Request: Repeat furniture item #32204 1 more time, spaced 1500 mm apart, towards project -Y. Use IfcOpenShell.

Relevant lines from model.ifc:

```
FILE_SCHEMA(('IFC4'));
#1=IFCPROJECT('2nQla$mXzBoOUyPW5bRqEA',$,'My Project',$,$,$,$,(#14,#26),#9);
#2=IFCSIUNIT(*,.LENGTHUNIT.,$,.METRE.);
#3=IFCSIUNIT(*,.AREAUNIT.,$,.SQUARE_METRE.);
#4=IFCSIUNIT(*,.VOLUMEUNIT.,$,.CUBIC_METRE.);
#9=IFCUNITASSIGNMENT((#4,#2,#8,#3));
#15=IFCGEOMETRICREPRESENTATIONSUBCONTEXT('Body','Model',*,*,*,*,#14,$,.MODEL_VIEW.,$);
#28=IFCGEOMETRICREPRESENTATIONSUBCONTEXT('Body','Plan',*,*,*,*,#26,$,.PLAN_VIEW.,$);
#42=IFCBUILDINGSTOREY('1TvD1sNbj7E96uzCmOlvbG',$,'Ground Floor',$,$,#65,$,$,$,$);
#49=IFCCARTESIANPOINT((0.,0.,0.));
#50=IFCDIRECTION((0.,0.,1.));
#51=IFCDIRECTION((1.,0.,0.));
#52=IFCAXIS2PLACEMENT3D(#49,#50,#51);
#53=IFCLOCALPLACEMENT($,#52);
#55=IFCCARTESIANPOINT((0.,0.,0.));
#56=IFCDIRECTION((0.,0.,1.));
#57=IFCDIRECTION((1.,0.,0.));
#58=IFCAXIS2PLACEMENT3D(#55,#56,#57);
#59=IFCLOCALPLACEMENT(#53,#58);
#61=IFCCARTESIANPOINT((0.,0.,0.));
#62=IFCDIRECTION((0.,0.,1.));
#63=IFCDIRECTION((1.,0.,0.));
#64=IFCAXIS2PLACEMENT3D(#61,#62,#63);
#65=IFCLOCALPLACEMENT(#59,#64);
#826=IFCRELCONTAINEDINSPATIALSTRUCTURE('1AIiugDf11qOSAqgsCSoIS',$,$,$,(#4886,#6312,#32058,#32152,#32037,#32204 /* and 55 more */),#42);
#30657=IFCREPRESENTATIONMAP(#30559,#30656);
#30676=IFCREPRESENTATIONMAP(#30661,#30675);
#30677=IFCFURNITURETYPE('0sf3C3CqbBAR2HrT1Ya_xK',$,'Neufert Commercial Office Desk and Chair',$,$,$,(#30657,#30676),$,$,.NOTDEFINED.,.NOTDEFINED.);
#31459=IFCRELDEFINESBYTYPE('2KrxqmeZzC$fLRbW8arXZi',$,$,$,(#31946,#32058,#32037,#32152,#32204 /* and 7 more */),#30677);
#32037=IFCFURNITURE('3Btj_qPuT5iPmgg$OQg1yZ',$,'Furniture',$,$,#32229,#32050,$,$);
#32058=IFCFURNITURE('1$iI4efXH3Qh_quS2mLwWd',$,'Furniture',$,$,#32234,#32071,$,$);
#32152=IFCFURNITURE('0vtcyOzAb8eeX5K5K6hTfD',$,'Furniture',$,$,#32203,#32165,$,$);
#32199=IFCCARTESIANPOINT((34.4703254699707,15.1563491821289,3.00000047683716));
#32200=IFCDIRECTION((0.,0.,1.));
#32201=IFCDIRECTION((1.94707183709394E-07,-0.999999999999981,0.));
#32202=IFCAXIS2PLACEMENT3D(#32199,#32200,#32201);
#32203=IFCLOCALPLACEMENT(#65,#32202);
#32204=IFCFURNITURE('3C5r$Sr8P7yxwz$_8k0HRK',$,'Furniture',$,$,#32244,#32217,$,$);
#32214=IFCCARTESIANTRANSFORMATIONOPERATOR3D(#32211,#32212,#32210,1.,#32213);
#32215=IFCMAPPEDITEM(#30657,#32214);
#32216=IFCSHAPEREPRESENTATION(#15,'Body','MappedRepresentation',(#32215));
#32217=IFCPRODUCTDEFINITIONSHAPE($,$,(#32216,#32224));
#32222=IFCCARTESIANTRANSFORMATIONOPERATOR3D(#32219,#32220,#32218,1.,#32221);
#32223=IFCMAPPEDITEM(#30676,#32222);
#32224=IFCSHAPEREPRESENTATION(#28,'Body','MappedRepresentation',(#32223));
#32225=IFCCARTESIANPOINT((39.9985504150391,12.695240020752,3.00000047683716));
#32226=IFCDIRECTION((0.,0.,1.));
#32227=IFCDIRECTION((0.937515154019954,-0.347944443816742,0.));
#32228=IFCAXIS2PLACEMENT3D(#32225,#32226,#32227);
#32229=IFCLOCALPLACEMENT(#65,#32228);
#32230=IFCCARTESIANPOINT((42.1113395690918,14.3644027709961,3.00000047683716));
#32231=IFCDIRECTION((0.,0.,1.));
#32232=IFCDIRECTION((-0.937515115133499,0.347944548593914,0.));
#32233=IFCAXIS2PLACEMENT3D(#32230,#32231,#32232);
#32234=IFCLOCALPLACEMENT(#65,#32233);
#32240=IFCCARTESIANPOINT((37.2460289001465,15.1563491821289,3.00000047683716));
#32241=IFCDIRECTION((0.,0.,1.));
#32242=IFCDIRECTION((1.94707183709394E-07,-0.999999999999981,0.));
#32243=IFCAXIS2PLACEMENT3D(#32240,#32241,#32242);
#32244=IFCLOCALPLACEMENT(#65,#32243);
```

```python
import numpy as np
import ifcopenshell
import ifcopenshell.api.geometry
import ifcopenshell.api.root
import ifcopenshell.util.element
import ifcopenshell.util.placement

model = ifcopenshell.open("model.ifc")

source = model.by_guid("3C5r$Sr8P7yxwz$_8k0HRK")
base = ifcopenshell.util.placement.get_local_placement(source.ObjectPlacement)
step = np.array([0.0, -1.0, 0.0]) * 1.5

for i in range(1, 2):
    copy = ifcopenshell.api.root.copy_class(model, product=source)
    copy.Representation = ifcopenshell.util.element.copy_deep(
        model, source.Representation, exclude=["IfcGeometricRepresentationContext", "IfcRepresentationMap"]
    )
    matrix = base.copy()
    matrix[:3, 3] += i * step
    print("added at", matrix[:3, 3].round(3) + 0.0)
    ifcopenshell.api.geometry.edit_object_placement(model, product=copy, matrix=matrix, is_si=False)

model.write("model_updated.ifc")
```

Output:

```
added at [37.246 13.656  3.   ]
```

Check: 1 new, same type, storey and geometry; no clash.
